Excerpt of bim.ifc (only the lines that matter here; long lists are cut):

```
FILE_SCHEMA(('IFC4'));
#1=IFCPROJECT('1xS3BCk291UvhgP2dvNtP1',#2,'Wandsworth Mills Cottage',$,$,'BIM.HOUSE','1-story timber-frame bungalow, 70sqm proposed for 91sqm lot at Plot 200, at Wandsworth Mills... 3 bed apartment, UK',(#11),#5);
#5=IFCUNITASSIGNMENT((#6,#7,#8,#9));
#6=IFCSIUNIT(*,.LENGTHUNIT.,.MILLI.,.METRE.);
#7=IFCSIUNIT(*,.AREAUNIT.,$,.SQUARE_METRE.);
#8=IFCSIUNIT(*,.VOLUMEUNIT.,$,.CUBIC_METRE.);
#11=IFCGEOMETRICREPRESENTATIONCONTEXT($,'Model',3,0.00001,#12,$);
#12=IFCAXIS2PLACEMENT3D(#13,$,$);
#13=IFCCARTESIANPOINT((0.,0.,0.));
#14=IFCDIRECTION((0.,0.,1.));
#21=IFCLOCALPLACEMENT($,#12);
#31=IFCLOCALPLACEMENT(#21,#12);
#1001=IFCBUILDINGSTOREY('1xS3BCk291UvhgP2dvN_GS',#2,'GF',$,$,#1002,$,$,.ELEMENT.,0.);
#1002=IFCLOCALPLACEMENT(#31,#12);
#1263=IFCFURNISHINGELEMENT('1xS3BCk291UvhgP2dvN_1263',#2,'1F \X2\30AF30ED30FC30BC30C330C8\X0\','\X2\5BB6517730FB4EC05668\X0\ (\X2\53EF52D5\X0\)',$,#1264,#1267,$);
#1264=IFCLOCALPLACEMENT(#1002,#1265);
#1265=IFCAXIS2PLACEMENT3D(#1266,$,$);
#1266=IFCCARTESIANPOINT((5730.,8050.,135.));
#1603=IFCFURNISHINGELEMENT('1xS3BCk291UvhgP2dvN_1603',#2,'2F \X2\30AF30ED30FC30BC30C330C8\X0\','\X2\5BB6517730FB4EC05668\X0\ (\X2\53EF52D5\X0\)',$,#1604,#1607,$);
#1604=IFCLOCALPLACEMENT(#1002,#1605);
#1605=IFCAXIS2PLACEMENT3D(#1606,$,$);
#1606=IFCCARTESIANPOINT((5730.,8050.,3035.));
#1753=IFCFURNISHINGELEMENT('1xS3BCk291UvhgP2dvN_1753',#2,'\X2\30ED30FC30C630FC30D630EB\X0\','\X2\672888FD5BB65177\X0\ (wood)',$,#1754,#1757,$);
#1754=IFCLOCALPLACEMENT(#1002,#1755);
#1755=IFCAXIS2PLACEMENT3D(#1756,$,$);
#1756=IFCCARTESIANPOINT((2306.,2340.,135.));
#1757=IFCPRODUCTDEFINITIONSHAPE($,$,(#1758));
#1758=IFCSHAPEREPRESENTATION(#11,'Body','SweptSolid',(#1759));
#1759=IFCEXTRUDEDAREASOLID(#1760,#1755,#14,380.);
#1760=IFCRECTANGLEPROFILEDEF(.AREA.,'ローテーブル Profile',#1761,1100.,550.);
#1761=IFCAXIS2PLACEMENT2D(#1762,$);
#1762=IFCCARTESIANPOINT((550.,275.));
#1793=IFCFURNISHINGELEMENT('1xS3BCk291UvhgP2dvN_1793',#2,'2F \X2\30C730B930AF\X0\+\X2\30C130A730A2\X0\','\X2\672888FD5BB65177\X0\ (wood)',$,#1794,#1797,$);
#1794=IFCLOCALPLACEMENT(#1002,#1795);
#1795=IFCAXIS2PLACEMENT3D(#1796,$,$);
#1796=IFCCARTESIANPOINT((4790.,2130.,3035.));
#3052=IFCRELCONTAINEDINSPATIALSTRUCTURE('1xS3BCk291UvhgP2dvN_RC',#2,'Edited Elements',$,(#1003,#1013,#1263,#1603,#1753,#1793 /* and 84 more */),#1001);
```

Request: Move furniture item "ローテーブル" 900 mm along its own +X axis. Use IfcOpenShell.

```python
import ifcopenshell
import ifcopenshell.api.geometry
import ifcopenshell.util.placement

model = ifcopenshell.open("bim.ifc")

item = model.by_id(1753)
matrix = ifcopenshell.util.placement.get_local_placement(item.ObjectPlacement)
matrix[:3, 3] += matrix[:3, 0] * 900.0
ifcopenshell.api.geometry.edit_object_placement(model, product=item, matrix=matrix, is_si=False)

print(ifcopenshell.util.placement.get_local_placement(item.ObjectPlacement).round(3) + 0.0)

model.write("bim-out.ifc")
```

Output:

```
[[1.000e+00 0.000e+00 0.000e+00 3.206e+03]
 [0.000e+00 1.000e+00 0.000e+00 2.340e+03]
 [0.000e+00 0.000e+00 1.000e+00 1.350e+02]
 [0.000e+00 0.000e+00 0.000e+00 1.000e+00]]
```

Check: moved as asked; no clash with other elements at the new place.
